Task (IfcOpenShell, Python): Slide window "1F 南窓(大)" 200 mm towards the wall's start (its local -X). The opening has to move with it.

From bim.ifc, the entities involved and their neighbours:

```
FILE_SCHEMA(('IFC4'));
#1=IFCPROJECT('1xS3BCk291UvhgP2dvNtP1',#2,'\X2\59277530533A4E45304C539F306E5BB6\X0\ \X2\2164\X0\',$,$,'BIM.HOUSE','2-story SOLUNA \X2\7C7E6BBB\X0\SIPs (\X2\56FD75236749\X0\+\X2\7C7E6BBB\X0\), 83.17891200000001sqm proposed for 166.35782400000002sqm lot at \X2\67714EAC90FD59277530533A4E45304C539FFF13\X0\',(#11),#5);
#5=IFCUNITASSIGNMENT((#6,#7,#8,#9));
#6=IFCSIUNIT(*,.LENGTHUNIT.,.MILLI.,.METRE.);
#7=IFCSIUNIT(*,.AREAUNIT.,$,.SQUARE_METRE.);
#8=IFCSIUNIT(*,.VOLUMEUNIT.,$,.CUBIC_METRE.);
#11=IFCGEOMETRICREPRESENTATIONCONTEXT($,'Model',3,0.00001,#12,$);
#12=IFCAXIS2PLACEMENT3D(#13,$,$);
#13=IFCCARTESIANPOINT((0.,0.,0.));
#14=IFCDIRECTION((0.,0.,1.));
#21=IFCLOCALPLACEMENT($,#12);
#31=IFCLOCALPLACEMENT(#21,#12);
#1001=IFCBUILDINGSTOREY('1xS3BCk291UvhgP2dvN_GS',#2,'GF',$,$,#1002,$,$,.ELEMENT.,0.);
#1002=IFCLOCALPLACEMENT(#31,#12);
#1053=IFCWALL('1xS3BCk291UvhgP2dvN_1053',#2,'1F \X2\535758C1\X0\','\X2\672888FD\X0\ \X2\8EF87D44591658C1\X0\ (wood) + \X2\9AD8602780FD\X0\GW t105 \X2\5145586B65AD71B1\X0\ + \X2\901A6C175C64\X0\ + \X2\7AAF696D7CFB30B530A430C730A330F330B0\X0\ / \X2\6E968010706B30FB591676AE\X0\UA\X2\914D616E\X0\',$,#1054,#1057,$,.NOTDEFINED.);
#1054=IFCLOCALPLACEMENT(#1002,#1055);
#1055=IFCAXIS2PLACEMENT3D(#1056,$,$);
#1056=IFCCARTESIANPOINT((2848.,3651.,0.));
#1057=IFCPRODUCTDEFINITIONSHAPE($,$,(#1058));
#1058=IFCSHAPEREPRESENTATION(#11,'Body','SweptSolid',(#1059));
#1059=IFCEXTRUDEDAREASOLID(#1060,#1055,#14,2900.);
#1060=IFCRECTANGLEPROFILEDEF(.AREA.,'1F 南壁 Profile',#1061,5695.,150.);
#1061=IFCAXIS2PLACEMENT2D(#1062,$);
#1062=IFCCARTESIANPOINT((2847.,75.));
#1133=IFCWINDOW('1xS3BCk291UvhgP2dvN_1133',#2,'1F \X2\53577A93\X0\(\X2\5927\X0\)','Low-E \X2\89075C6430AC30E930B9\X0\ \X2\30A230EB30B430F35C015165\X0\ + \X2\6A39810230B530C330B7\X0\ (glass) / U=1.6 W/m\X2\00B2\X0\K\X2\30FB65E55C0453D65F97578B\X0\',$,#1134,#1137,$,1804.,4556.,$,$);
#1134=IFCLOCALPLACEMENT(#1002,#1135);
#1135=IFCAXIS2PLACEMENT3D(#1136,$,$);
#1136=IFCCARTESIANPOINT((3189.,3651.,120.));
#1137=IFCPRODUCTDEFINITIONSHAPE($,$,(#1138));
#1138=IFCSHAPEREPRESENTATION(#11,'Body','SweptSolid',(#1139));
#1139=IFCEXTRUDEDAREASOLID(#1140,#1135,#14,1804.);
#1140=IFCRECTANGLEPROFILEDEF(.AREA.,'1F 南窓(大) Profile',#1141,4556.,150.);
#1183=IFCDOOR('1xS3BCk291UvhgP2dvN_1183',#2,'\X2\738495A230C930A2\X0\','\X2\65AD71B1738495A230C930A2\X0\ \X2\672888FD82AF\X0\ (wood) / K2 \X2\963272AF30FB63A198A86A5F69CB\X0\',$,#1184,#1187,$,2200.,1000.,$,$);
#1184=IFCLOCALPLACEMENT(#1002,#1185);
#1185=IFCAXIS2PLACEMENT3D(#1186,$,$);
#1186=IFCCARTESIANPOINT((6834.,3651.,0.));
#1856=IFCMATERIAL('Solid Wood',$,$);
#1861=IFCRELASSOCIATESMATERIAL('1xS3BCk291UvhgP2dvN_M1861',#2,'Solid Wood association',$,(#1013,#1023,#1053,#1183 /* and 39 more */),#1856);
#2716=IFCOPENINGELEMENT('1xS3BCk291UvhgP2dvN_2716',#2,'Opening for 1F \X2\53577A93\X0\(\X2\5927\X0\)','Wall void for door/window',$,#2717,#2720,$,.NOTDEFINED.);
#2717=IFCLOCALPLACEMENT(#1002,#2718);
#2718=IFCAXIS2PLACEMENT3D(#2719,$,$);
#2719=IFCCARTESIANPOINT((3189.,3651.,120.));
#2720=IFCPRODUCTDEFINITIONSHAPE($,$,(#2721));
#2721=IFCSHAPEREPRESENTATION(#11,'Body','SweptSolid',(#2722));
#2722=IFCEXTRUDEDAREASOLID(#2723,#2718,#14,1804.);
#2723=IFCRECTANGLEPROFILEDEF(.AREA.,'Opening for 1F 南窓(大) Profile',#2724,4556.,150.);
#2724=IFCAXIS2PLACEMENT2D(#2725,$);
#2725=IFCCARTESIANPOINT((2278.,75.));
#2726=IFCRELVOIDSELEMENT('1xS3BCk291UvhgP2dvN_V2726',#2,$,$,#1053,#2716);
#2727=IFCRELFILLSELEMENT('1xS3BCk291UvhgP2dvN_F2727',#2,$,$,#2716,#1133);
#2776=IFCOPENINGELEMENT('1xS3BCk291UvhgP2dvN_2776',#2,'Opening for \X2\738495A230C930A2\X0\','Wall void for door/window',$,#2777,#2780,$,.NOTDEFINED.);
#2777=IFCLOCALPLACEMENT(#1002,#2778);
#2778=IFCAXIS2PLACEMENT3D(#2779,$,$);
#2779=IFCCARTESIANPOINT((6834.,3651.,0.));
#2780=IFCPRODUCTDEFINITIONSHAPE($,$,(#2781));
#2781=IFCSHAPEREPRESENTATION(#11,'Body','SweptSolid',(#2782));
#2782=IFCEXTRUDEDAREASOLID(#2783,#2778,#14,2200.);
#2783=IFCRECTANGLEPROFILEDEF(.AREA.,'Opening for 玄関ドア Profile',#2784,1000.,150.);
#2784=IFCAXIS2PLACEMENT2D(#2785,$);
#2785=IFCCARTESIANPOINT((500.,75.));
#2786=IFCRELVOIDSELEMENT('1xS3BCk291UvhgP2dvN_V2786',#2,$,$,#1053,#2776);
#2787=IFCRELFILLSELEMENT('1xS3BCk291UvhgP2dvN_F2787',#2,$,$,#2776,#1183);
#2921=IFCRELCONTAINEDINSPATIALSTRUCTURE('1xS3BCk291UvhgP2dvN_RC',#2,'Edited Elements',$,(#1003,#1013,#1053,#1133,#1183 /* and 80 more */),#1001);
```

```python
import ifcopenshell
import ifcopenshell.api.geometry
import ifcopenshell.util.placement

model = ifcopenshell.open("bim.ifc")

window = model.by_guid("1xS3BCk291UvhgP2dvN_1133")
opening = window.FillsVoids[0].RelatingOpeningElement
wall = opening.VoidsElements[0].RelatingBuildingElement

wall_matrix = ifcopenshell.util.placement.get_local_placement(wall.ObjectPlacement)
shift = wall_matrix[:3, 0] * -200.0
before = ifcopenshell.util.placement.get_local_placement(window.ObjectPlacement)[:3, 3].copy()

# The window is not placed relative to its opening, so move both.
for product in (opening, window):
    matrix = ifcopenshell.util.placement.get_local_placement(product.ObjectPlacement)
    matrix[:3, 3] += shift
    ifcopenshell.api.geometry.edit_object_placement(model, product=product, matrix=matrix, is_si=False)

after = ifcopenshell.util.placement.get_local_placement(window.ObjectPlacement)[:3, 3]
print("window moved by", (after - before).round(3) + 0.0)

model.write("bim_rev.ifc")
```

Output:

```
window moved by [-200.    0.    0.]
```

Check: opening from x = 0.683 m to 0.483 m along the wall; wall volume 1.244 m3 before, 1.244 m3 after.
